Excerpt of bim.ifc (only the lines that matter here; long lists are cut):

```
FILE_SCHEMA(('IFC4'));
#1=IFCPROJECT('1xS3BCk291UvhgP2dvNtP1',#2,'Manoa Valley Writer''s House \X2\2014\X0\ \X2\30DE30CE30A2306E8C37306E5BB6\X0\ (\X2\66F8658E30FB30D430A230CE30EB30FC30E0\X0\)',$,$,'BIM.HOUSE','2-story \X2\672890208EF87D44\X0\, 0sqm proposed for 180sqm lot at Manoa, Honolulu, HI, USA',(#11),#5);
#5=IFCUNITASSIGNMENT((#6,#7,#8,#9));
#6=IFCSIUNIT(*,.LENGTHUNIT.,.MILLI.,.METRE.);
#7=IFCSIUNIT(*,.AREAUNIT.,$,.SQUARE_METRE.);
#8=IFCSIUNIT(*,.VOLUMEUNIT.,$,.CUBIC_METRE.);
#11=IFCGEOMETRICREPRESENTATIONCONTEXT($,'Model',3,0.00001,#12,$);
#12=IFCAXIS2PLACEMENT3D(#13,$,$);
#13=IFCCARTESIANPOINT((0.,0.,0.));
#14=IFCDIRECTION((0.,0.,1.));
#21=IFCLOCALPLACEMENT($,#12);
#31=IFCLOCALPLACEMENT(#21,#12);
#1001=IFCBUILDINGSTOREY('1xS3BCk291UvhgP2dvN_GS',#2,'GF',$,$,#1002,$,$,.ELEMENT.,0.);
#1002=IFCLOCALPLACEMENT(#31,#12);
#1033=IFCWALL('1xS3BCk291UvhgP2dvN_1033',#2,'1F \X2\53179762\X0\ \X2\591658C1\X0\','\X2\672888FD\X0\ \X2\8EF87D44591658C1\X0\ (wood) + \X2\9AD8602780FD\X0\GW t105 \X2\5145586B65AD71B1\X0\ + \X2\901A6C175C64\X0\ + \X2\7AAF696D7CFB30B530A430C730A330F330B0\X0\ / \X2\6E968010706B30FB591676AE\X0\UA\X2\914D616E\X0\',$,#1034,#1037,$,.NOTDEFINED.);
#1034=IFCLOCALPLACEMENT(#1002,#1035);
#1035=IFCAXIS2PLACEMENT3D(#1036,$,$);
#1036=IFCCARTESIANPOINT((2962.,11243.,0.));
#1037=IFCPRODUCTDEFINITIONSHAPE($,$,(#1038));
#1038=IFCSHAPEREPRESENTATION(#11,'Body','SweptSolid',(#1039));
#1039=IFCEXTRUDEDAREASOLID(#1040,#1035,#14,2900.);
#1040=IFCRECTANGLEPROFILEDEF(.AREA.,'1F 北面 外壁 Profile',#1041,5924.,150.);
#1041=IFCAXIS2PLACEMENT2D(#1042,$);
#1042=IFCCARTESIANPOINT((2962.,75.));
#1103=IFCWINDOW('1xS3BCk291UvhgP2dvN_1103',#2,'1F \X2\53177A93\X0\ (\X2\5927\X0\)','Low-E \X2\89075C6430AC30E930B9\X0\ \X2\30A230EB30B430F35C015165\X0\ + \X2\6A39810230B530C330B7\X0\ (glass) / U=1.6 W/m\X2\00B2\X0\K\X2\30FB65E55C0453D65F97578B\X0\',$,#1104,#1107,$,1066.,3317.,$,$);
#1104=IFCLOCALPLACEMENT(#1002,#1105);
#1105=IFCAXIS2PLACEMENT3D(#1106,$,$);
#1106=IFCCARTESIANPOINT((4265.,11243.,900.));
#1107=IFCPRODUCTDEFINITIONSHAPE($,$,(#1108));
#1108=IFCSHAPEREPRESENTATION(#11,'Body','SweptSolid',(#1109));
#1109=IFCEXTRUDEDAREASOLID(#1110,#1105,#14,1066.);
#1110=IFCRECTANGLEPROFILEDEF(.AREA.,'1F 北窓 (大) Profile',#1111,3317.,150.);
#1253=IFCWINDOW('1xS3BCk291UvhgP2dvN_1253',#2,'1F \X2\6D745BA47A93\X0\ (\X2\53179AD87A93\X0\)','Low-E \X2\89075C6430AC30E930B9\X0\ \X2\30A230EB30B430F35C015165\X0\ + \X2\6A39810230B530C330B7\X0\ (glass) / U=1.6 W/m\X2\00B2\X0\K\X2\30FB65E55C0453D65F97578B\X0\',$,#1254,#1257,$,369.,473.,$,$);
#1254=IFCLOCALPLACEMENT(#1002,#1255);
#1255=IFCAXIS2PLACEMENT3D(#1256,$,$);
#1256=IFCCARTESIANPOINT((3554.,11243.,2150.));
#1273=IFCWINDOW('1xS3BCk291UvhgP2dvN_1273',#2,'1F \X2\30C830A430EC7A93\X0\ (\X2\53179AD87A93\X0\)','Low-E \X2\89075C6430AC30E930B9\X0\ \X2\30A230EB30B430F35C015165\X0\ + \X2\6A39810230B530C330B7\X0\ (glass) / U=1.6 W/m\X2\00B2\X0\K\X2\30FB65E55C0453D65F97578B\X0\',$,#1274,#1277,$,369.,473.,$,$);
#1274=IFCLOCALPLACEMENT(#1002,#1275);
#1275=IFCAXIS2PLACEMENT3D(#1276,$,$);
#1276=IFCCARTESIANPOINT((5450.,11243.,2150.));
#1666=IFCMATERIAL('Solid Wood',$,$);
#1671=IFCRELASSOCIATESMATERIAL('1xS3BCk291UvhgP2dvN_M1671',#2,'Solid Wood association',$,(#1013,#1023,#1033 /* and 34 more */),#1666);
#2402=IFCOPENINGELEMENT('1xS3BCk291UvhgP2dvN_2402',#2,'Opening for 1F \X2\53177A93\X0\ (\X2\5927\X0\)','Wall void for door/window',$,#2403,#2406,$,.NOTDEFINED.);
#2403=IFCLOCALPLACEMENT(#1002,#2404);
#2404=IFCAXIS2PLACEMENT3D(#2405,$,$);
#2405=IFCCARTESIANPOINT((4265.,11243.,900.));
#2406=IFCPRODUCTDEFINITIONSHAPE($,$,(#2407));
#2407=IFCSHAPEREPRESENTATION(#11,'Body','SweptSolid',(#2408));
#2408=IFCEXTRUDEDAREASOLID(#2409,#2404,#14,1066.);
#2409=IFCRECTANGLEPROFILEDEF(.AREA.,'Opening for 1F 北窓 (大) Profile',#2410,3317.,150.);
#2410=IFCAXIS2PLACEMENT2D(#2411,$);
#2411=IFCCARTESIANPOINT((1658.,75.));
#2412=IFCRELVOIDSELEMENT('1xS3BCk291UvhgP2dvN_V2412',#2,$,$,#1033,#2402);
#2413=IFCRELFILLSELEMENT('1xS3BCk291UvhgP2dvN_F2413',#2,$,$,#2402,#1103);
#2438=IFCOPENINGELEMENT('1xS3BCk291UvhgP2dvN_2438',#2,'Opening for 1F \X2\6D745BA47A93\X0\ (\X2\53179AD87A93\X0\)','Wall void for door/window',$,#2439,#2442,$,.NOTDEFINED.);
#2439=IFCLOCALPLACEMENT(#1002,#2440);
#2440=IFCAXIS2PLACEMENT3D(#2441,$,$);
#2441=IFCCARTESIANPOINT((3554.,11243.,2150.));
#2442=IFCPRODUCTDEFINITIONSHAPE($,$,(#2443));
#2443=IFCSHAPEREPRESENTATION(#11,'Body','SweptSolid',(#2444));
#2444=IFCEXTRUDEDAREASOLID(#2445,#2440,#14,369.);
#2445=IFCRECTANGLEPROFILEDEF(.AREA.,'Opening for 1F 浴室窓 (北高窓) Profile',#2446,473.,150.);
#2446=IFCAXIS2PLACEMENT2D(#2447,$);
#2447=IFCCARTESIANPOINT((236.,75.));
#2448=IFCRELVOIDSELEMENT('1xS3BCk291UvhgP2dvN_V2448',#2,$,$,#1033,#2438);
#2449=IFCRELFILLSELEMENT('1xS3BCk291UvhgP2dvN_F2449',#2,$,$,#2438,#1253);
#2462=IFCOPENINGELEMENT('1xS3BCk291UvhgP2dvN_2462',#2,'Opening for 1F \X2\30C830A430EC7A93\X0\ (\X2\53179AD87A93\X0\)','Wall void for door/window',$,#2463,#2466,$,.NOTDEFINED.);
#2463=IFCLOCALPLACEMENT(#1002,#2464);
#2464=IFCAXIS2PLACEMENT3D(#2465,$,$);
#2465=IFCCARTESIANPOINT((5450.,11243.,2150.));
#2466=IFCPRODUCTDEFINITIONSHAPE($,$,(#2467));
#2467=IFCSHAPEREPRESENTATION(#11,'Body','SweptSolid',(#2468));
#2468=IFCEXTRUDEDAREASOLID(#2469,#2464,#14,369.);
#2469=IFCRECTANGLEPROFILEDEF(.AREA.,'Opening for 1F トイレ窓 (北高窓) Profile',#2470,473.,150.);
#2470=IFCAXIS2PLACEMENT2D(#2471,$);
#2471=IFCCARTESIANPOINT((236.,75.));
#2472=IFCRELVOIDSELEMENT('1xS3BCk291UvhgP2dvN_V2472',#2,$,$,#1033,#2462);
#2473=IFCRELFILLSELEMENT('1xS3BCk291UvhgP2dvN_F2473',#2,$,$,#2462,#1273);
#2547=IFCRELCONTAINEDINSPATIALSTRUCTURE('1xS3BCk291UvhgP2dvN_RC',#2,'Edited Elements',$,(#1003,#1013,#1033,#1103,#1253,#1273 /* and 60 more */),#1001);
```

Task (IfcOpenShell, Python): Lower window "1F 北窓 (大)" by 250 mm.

```python
import numpy as np
import ifcopenshell
import ifcopenshell.api.geometry
import ifcopenshell.util.placement
import ifcopenshell.util.unit

model = ifcopenshell.open("bim.ifc")
unit_scale = ifcopenshell.util.unit.calculate_unit_scale(model)

window = model.by_guid("1xS3BCk291UvhgP2dvN_1103")
opening = window.FillsVoids[0].RelatingOpeningElement
dz = -0.25 / unit_scale

shift = np.array([0.0, 0.0, dz])
# The window is not placed relative to its opening, so move both.
for product in (opening, window):
    matrix = ifcopenshell.util.placement.get_local_placement(product.ObjectPlacement)
    matrix[:3, 3] += shift
    ifcopenshell.api.geometry.edit_object_placement(model, product=product, matrix=matrix, is_si=False)

print(f"moved by {dz * unit_scale:+.3f} m")

model.write("bim_edited.ifc")
```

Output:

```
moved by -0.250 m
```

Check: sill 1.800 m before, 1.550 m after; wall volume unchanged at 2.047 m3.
